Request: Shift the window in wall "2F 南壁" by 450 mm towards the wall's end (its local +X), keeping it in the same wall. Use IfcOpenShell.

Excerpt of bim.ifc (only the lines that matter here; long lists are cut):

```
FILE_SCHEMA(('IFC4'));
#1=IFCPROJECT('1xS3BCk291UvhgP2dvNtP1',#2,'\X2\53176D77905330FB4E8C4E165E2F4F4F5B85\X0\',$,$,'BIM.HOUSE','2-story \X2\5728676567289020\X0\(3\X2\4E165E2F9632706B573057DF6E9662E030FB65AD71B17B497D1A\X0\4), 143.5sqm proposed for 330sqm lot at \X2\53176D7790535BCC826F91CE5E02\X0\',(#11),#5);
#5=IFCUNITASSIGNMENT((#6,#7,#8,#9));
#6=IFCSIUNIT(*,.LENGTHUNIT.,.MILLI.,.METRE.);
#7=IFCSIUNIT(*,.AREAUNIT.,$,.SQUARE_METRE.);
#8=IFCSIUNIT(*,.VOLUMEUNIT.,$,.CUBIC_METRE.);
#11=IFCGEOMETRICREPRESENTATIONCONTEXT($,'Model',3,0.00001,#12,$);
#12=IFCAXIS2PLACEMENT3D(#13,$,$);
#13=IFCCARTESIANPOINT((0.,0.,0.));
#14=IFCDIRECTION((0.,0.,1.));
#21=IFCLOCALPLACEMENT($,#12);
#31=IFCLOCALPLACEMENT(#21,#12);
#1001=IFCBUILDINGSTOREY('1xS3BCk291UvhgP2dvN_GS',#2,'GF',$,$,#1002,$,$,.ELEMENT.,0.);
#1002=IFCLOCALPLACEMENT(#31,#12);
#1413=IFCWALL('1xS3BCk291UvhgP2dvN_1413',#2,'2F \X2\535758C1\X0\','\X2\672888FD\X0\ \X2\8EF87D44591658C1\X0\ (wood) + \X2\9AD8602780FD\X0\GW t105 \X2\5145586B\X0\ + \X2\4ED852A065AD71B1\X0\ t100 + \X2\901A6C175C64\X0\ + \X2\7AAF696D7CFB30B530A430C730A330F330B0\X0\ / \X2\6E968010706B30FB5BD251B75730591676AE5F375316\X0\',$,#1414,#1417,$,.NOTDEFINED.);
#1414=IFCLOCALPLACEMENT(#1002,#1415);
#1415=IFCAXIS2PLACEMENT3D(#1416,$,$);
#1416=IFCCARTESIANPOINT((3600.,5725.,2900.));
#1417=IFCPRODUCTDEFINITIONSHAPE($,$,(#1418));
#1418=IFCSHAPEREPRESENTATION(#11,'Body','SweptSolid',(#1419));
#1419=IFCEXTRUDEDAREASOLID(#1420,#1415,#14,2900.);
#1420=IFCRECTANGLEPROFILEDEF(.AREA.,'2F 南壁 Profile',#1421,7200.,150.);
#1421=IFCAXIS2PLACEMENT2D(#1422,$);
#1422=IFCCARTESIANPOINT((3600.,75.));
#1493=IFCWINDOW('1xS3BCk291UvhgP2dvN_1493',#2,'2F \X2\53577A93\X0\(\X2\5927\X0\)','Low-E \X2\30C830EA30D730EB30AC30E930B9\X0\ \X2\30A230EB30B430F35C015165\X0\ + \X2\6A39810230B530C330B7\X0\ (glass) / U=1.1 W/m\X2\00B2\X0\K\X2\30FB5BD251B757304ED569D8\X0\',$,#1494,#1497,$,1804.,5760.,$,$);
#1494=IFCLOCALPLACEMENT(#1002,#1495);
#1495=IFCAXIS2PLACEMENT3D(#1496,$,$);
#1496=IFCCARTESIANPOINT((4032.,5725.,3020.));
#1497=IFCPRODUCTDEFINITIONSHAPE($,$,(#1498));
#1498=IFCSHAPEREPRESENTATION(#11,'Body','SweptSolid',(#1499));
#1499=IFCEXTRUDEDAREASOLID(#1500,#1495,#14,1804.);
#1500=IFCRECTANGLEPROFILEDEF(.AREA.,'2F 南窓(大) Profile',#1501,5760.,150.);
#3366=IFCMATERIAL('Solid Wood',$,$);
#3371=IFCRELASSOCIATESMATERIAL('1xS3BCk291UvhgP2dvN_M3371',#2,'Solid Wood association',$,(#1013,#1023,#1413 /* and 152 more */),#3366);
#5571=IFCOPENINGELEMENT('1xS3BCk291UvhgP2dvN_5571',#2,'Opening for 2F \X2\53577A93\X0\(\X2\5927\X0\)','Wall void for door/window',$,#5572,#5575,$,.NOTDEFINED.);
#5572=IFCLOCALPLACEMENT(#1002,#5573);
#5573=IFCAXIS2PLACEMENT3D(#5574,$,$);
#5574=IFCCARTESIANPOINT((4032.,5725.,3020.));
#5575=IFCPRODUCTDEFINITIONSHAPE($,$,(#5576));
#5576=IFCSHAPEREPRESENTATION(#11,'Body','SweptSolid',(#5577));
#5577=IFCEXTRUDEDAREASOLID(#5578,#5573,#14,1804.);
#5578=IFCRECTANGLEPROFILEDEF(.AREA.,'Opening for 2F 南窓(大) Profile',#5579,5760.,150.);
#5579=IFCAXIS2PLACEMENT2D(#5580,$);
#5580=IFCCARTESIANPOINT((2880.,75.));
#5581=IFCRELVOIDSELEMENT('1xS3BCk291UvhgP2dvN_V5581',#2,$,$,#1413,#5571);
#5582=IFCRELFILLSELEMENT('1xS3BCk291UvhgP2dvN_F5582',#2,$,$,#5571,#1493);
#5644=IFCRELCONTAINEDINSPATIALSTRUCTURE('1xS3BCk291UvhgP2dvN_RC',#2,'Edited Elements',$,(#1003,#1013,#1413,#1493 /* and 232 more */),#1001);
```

```python
import ifcopenshell
import ifcopenshell.api.geometry
import ifcopenshell.util.placement

model = ifcopenshell.open("bim.ifc")

window = model.by_guid("1xS3BCk291UvhgP2dvN_1493")
opening = window.FillsVoids[0].RelatingOpeningElement
wall = opening.VoidsElements[0].RelatingBuildingElement

wall_matrix = ifcopenshell.util.placement.get_local_placement(wall.ObjectPlacement)
shift = wall_matrix[:3, 0] * 450.0
before = ifcopenshell.util.placement.get_local_placement(window.ObjectPlacement)[:3, 3].copy()

# The window is not placed relative to its opening, so move both.
for product in (opening, window):
    matrix = ifcopenshell.util.placement.get_local_placement(product.ObjectPlacement)
    matrix[:3, 3] += shift
    ifcopenshell.api.geometry.edit_object_placement(model, product=product, matrix=matrix, is_si=False)

after = ifcopenshell.util.placement.get_local_placement(window.ObjectPlacement)[:3, 3]
print("window moved by", (after - before).round(3) + 0.0)

model.write("bim_rev.ifc")
```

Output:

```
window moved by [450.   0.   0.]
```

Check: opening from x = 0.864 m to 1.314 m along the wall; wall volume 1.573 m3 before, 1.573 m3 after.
